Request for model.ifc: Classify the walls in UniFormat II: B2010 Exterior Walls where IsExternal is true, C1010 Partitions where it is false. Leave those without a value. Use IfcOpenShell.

First a look at what the model holds.

```python
import ifcopenshell
import ifcopenshell.util.element

model = ifcopenshell.open("model.ifc")
print(model.schema)
print("classifications:", [c.Name for c in model.by_type("IfcClassification")])
values = [ifcopenshell.util.element.get_pset(e, "Pset_WallCommon", "IsExternal") for e in model.by_type("IfcWall")]
for value in (True, False, None):
    print("IsExternal", value, values.count(value))
```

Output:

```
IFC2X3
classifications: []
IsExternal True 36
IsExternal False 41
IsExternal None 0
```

```python
import ifcopenshell
import ifcopenshell.api.classification
import ifcopenshell.util.element

model = ifcopenshell.open("model.ifc")

# IFC2X3 requires Source and Edition and has no link from the project to the system.
system = model.create_entity("IfcClassification", Source="ASTM", Edition="E1557", Name="UniFormat II")

walls = model.by_type("IfcWall")
external = {e: ifcopenshell.util.element.get_pset(e, "Pset_WallCommon", "IsExternal") for e in walls}
for flag, code, name in ((True, "B2010", "Exterior Walls"), (False, "C1010", "Partitions")):
    products = [e for e in walls if external[e] is flag]
    ifcopenshell.api.classification.add_reference(
        model, products=products, classification=system, identification=code, name=name
    )
    print(code, len(products))

model.write("model_v2.ifc")
```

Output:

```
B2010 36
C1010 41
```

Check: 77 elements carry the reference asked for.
